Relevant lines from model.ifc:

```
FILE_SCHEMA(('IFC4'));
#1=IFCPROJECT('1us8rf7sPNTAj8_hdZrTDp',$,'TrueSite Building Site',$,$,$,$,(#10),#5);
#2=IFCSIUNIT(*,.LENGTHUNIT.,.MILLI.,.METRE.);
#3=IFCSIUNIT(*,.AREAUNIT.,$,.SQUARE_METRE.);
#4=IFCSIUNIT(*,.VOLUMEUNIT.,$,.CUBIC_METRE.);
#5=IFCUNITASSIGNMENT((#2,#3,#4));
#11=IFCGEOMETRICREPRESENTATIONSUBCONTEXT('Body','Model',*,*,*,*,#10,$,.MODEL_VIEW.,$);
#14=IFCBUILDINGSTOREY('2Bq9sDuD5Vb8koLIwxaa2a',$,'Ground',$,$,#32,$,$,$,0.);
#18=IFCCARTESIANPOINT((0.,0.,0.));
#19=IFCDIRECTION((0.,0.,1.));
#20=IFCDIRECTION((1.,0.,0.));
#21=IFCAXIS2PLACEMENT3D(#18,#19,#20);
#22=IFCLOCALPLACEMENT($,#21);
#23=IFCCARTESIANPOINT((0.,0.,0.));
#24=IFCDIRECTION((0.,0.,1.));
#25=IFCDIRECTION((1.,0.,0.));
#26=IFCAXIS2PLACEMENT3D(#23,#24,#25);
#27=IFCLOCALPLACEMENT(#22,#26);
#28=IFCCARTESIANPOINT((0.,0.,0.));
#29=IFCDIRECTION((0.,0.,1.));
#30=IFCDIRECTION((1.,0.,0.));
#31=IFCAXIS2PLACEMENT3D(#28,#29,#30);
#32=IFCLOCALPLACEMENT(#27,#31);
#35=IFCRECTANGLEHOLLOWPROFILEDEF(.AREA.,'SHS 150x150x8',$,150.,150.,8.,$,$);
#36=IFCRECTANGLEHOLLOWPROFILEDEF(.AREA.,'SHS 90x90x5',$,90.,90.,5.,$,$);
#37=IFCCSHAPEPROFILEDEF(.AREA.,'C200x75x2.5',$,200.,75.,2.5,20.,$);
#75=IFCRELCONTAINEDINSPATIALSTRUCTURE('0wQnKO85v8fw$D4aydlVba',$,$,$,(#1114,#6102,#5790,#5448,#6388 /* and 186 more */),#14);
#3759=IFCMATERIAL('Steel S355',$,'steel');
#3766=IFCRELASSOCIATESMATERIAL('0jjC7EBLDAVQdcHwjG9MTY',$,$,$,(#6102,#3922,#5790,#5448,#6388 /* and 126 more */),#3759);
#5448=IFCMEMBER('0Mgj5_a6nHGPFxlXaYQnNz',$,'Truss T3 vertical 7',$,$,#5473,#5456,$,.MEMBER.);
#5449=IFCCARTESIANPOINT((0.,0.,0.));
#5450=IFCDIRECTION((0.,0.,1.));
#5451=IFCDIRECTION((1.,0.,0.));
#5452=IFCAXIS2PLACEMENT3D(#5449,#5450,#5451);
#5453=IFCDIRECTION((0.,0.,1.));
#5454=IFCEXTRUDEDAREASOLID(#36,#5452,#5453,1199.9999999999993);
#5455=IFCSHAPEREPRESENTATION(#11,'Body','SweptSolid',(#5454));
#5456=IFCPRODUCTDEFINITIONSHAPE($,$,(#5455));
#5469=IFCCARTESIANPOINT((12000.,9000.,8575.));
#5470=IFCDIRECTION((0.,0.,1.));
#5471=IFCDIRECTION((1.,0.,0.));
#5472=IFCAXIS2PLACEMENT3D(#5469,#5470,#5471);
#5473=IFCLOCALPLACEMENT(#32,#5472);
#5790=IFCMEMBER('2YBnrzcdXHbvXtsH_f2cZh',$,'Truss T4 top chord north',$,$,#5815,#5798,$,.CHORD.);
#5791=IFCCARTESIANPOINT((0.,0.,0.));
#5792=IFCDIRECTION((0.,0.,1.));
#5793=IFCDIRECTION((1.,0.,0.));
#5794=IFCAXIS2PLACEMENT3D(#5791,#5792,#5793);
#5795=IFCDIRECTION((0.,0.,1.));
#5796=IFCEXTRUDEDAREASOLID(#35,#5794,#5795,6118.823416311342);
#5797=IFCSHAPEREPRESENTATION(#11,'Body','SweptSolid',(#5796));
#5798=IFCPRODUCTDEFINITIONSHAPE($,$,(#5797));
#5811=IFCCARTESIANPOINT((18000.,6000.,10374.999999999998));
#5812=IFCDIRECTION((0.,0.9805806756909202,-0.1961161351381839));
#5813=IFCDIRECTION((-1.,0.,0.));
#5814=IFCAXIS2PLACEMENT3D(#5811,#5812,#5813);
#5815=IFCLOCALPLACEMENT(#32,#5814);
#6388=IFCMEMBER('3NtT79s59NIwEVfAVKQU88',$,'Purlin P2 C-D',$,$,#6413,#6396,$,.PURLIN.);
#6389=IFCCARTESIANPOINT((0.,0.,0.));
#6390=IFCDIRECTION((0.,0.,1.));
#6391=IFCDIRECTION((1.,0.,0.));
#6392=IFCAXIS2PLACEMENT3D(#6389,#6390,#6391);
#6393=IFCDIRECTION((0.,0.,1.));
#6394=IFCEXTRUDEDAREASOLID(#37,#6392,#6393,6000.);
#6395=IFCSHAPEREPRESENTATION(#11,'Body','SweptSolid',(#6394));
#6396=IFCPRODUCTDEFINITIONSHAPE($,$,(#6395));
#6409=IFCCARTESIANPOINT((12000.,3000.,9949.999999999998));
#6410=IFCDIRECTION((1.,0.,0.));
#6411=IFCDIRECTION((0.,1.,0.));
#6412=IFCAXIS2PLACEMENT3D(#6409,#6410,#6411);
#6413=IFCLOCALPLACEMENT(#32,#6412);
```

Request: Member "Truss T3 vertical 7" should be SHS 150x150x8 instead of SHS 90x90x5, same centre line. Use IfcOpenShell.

```python
import ifcopenshell
import ifcopenshell.util.element
import ifcopenshell.util.representation

model = ifcopenshell.open("model.ifc")

member = model.by_guid("0Mgj5_a6nHGPFxlXaYQnNz")
source = next(p for p in model.by_type("IfcRectangleHollowProfileDef") if p.ProfileName == "SHS 150x150x8")

body = ifcopenshell.util.representation.get_representation(member, "Model", "Body")
solid = body.Items[0]
old_profile = solid.SweptArea

# Copy the section's sizes but keep this member's own profile position.
profile = ifcopenshell.util.element.copy(model, source)
profile.Position = old_profile.Position
solid.SweptArea = profile
if not model.get_total_inverses(old_profile):
    ifcopenshell.util.element.remove_deep2(model, old_profile)

print(solid.SweptArea)

model.write("model_edited.ifc")
```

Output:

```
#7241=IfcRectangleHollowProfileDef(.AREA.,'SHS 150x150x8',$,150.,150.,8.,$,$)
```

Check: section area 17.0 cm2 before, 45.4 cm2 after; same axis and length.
